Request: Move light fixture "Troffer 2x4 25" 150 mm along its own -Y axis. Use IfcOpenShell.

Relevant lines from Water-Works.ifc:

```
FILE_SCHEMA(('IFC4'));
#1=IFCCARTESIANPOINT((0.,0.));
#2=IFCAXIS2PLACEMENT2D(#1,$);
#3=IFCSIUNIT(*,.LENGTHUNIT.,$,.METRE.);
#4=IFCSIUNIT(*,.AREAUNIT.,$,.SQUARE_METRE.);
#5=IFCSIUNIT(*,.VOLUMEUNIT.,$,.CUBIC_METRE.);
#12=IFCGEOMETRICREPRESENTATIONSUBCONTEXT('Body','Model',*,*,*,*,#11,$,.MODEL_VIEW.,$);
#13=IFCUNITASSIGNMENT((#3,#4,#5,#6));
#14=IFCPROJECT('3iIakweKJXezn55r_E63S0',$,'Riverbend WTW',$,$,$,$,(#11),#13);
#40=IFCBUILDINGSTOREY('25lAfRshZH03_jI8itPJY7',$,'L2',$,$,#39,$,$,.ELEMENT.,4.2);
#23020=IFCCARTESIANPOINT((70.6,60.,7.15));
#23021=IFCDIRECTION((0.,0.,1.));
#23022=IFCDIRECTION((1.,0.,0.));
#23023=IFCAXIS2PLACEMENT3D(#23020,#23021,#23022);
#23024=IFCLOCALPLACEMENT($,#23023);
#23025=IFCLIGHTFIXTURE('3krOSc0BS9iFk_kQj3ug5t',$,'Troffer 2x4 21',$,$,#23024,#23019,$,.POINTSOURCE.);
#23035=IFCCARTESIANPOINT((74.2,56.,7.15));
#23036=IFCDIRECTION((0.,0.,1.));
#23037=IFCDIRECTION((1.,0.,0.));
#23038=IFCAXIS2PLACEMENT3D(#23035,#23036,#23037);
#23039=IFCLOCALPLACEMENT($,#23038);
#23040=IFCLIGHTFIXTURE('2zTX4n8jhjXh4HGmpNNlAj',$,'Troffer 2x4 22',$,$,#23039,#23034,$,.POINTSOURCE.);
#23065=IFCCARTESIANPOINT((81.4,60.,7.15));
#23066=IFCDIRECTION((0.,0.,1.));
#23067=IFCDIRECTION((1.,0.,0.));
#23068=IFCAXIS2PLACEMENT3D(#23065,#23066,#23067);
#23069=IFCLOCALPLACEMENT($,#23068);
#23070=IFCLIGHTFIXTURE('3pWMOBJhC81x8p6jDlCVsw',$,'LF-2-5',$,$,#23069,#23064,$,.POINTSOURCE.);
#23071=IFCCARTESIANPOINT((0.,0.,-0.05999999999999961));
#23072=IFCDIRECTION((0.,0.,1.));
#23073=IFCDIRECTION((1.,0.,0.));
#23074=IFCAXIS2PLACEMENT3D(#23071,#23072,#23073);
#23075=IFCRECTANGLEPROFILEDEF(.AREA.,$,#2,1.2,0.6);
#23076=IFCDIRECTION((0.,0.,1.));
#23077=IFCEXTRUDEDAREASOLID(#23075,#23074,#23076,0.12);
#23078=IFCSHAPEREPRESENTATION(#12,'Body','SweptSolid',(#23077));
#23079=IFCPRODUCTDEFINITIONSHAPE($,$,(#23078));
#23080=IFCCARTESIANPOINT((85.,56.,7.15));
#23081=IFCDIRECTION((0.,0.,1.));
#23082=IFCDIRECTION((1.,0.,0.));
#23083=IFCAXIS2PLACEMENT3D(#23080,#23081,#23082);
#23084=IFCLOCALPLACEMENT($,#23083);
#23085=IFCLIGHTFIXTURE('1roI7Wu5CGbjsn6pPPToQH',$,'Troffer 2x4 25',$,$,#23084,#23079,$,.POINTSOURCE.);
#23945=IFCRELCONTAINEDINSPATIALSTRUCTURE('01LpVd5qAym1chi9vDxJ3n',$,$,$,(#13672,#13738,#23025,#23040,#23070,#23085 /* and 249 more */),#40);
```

```python
import ifcopenshell
import ifcopenshell.api.geometry
import ifcopenshell.util.placement
import ifcopenshell.util.unit

model = ifcopenshell.open("Water-Works.ifc")
unit_scale = ifcopenshell.util.unit.calculate_unit_scale(model)

item = model.by_guid("1roI7Wu5CGbjsn6pPPToQH")
matrix = ifcopenshell.util.placement.get_local_placement(item.ObjectPlacement)
matrix[:3, 3] -= matrix[:3, 1] * 0.15 / unit_scale
ifcopenshell.api.geometry.edit_object_placement(model, product=item, matrix=matrix, is_si=False)

print(ifcopenshell.util.placement.get_local_placement(item.ObjectPlacement).round(3) + 0.0)

model.write("Water-Works_updated.ifc")
```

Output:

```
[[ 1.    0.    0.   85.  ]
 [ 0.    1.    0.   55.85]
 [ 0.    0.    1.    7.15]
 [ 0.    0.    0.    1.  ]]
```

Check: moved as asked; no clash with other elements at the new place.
